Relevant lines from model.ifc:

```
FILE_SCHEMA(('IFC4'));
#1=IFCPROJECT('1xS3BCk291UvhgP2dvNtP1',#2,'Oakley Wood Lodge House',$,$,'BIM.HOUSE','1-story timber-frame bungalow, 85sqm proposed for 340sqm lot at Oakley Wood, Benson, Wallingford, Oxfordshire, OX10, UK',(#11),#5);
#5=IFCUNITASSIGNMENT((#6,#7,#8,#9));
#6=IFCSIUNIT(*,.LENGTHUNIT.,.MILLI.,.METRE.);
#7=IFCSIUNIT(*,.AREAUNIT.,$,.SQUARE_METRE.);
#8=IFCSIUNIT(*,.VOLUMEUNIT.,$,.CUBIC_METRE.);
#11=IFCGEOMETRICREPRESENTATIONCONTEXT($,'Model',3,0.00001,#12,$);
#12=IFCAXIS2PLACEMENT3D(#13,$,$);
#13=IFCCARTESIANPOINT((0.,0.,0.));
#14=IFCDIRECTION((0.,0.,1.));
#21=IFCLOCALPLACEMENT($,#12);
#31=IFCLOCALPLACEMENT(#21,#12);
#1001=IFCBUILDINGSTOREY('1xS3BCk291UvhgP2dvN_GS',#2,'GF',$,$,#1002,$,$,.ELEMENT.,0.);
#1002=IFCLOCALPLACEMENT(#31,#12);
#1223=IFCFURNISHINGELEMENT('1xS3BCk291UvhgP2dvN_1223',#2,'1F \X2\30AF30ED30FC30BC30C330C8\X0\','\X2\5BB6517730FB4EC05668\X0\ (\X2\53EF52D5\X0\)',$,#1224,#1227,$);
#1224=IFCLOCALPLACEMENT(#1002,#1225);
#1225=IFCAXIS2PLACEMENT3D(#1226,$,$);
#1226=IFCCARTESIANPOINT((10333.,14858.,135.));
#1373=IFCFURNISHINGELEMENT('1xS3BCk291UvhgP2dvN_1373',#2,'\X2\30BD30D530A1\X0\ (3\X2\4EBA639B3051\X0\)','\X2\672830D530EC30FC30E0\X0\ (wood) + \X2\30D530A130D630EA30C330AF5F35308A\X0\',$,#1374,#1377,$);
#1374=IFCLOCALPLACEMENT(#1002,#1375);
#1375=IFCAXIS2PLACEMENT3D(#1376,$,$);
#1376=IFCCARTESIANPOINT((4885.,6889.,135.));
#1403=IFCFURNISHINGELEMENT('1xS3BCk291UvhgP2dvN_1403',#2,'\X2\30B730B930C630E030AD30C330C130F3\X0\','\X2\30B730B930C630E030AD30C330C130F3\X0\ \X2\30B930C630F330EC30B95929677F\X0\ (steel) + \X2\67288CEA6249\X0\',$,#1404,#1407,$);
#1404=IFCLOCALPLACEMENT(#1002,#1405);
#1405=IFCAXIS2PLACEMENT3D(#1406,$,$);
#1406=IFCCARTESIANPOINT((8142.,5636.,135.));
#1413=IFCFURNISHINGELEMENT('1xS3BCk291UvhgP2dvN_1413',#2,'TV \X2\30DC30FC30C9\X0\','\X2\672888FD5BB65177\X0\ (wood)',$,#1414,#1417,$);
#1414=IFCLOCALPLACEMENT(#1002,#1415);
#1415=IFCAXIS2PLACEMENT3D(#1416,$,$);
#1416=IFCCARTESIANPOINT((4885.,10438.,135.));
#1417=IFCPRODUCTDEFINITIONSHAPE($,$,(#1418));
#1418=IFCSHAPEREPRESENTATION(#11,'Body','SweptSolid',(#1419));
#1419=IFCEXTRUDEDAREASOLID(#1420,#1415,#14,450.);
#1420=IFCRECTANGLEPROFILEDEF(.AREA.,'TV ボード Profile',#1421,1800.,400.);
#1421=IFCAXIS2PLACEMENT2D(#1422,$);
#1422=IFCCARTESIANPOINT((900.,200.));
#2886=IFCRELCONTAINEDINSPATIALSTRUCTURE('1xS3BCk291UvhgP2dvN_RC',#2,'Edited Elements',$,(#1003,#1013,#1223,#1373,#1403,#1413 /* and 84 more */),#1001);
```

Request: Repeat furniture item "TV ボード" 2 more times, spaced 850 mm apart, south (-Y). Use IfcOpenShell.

```python
import numpy as np
import ifcopenshell
import ifcopenshell.api.geometry
import ifcopenshell.api.root
import ifcopenshell.util.element
import ifcopenshell.util.placement

model = ifcopenshell.open("model.ifc")


def reuse_history(source, copy):
    """copy_class also copies each property set's owner history, people and application; keep the originals."""
    for rel in copy.IsDefinedBy:
        if rel.is_a("IfcRelDefinesByProperties") and (history := rel.RelatingPropertyDefinition.OwnerHistory):
            rel.RelatingPropertyDefinition.OwnerHistory = source.OwnerHistory
            ifcopenshell.util.element.remove_deep2(model, history)


source = model.by_guid("1xS3BCk291UvhgP2dvN_1413")
base = ifcopenshell.util.placement.get_local_placement(source.ObjectPlacement)
step = np.array([0.0, -1.0, 0.0]) * 850.0

for i in range(1, 3):
    copy = ifcopenshell.api.root.copy_class(model, product=source)
    copy.Representation = ifcopenshell.util.element.copy_deep(
        model, source.Representation, exclude=["IfcGeometricRepresentationContext", "IfcRepresentationMap"]
    )
    reuse_history(source, copy)
    matrix = base.copy()
    matrix[:3, 3] += i * step
    print("added at", matrix[:3, 3].round(3) + 0.0)
    ifcopenshell.api.geometry.edit_object_placement(model, product=copy, matrix=matrix, is_si=False)

model.write("model-out.ifc")
```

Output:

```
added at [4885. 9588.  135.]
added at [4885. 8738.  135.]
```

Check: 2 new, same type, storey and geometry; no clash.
